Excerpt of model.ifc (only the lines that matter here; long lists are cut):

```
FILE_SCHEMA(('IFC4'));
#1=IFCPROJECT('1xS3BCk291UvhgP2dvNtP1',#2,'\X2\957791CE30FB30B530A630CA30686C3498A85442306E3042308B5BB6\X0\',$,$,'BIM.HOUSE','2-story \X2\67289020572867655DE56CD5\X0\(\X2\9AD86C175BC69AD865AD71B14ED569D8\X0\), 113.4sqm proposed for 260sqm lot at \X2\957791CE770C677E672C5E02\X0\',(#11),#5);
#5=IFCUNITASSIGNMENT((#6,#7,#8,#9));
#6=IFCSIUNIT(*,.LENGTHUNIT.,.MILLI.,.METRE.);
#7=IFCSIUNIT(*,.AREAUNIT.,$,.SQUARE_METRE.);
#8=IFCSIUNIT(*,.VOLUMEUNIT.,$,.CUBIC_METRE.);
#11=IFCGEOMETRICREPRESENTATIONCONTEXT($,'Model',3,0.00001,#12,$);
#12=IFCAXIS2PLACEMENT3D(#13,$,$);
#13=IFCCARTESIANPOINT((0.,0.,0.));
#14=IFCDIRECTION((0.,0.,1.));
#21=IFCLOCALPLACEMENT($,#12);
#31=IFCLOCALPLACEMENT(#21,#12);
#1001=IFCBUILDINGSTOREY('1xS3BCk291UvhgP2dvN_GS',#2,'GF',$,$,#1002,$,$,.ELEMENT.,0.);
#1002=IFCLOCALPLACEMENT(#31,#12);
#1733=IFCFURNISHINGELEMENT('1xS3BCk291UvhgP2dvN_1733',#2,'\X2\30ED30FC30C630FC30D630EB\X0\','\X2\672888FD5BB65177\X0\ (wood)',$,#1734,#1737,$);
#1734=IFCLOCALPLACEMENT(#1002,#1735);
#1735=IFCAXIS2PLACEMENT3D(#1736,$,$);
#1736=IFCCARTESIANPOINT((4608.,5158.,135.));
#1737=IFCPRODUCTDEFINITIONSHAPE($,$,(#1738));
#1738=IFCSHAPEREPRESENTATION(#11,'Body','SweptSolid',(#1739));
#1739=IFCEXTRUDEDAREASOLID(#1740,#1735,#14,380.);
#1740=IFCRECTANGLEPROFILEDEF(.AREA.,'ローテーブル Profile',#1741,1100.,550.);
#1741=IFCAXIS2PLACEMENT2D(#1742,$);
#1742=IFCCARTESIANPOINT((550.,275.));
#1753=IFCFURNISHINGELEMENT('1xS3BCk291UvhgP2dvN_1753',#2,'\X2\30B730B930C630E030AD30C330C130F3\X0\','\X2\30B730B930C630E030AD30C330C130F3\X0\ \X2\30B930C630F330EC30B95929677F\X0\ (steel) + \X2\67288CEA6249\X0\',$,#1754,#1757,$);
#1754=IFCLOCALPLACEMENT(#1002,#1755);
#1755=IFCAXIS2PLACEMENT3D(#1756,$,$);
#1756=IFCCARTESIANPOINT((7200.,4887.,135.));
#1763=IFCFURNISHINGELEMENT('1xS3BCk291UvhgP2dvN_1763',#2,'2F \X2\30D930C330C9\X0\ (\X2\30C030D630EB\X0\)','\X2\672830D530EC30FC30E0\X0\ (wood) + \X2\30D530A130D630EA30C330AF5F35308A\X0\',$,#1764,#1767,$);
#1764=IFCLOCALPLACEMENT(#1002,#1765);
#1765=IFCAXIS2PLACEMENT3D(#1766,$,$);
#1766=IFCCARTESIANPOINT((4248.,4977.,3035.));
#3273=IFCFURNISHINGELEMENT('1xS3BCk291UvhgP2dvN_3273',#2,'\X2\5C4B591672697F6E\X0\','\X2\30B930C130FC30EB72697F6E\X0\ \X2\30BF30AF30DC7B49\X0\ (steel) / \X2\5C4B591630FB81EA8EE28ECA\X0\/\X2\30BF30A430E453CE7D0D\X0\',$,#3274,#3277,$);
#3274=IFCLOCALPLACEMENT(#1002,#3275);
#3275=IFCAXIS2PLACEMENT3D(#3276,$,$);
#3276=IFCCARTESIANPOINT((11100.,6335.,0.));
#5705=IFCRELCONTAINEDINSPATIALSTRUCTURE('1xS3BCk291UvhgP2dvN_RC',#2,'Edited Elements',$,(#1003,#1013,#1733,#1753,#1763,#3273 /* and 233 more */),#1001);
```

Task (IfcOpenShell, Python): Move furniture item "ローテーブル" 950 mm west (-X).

```python
import ifcopenshell
import ifcopenshell.api.geometry
import ifcopenshell.util.placement

model = ifcopenshell.open("model.ifc")

item = model.by_guid("1xS3BCk291UvhgP2dvN_1733")
matrix = ifcopenshell.util.placement.get_local_placement(item.ObjectPlacement)
matrix[0, 3] -= 950.0
ifcopenshell.api.geometry.edit_object_placement(model, product=item, matrix=matrix, is_si=False)

print(ifcopenshell.util.placement.get_local_placement(item.ObjectPlacement).round(3) + 0.0)

model.write("model_edited.ifc")
```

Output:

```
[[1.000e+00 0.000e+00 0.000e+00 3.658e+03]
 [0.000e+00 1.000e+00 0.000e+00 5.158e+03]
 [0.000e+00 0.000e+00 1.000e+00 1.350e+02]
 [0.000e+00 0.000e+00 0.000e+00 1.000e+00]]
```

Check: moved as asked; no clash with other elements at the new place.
